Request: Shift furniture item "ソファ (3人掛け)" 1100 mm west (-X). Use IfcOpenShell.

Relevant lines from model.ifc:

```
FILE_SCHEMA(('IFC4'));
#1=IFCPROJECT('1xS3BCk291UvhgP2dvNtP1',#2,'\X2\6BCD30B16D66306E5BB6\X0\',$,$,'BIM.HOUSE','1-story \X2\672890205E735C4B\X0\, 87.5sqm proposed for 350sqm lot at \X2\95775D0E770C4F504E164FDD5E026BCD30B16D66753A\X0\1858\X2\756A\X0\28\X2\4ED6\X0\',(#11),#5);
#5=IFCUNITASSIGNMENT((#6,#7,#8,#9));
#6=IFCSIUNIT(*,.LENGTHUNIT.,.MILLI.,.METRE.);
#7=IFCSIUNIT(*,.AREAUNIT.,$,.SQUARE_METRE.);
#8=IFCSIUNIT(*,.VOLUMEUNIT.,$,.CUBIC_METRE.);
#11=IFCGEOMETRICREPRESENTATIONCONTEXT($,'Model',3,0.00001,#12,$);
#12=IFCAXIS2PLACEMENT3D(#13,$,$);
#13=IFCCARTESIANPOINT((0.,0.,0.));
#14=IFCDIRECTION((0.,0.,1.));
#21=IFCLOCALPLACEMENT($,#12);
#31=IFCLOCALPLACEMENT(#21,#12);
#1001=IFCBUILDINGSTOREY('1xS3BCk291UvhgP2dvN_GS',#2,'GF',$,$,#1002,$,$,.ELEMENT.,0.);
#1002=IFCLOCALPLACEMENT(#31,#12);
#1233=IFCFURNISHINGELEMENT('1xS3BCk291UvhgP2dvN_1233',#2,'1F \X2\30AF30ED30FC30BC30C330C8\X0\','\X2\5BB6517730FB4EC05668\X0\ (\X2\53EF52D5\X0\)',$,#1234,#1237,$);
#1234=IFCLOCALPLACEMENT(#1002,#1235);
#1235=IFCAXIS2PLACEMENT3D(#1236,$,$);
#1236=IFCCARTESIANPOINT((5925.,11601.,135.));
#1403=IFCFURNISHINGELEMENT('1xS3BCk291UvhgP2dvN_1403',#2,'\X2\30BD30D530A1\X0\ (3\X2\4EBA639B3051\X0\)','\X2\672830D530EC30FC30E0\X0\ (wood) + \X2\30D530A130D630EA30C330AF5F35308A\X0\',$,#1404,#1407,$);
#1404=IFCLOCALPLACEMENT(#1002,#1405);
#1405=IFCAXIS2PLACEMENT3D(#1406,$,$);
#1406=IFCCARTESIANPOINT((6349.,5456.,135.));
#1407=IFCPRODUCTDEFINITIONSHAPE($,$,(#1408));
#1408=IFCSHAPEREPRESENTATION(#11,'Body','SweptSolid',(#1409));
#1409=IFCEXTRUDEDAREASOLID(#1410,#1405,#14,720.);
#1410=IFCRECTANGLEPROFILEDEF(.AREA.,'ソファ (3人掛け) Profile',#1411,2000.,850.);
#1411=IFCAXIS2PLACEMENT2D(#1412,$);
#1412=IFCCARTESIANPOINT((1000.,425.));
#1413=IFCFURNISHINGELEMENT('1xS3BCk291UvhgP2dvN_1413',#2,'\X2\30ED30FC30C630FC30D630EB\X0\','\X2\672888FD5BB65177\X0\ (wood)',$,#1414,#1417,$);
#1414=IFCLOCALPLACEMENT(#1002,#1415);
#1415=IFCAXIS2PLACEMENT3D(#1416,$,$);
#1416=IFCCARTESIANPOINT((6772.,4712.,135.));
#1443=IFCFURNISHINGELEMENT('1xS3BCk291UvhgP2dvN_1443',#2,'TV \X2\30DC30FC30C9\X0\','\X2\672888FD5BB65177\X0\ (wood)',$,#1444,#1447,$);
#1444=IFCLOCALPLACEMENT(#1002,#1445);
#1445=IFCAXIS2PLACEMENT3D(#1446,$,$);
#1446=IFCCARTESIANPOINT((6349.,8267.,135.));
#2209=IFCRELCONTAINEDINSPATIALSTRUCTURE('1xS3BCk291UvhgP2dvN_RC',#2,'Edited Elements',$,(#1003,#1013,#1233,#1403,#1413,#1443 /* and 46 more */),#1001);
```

```python
import ifcopenshell
import ifcopenshell.api.geometry
import ifcopenshell.util.placement

model = ifcopenshell.open("model.ifc")

item = model.by_id(1403)
matrix = ifcopenshell.util.placement.get_local_placement(item.ObjectPlacement)
matrix[0, 3] -= 1100.0
ifcopenshell.api.geometry.edit_object_placement(model, product=item, matrix=matrix, is_si=False)

print(ifcopenshell.util.placement.get_local_placement(item.ObjectPlacement).round(3) + 0.0)

model.write("model_updated.ifc")
```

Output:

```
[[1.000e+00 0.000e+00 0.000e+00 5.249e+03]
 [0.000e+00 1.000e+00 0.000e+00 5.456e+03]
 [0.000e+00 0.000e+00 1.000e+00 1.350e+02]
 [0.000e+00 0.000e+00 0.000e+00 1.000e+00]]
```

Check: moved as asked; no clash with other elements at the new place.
